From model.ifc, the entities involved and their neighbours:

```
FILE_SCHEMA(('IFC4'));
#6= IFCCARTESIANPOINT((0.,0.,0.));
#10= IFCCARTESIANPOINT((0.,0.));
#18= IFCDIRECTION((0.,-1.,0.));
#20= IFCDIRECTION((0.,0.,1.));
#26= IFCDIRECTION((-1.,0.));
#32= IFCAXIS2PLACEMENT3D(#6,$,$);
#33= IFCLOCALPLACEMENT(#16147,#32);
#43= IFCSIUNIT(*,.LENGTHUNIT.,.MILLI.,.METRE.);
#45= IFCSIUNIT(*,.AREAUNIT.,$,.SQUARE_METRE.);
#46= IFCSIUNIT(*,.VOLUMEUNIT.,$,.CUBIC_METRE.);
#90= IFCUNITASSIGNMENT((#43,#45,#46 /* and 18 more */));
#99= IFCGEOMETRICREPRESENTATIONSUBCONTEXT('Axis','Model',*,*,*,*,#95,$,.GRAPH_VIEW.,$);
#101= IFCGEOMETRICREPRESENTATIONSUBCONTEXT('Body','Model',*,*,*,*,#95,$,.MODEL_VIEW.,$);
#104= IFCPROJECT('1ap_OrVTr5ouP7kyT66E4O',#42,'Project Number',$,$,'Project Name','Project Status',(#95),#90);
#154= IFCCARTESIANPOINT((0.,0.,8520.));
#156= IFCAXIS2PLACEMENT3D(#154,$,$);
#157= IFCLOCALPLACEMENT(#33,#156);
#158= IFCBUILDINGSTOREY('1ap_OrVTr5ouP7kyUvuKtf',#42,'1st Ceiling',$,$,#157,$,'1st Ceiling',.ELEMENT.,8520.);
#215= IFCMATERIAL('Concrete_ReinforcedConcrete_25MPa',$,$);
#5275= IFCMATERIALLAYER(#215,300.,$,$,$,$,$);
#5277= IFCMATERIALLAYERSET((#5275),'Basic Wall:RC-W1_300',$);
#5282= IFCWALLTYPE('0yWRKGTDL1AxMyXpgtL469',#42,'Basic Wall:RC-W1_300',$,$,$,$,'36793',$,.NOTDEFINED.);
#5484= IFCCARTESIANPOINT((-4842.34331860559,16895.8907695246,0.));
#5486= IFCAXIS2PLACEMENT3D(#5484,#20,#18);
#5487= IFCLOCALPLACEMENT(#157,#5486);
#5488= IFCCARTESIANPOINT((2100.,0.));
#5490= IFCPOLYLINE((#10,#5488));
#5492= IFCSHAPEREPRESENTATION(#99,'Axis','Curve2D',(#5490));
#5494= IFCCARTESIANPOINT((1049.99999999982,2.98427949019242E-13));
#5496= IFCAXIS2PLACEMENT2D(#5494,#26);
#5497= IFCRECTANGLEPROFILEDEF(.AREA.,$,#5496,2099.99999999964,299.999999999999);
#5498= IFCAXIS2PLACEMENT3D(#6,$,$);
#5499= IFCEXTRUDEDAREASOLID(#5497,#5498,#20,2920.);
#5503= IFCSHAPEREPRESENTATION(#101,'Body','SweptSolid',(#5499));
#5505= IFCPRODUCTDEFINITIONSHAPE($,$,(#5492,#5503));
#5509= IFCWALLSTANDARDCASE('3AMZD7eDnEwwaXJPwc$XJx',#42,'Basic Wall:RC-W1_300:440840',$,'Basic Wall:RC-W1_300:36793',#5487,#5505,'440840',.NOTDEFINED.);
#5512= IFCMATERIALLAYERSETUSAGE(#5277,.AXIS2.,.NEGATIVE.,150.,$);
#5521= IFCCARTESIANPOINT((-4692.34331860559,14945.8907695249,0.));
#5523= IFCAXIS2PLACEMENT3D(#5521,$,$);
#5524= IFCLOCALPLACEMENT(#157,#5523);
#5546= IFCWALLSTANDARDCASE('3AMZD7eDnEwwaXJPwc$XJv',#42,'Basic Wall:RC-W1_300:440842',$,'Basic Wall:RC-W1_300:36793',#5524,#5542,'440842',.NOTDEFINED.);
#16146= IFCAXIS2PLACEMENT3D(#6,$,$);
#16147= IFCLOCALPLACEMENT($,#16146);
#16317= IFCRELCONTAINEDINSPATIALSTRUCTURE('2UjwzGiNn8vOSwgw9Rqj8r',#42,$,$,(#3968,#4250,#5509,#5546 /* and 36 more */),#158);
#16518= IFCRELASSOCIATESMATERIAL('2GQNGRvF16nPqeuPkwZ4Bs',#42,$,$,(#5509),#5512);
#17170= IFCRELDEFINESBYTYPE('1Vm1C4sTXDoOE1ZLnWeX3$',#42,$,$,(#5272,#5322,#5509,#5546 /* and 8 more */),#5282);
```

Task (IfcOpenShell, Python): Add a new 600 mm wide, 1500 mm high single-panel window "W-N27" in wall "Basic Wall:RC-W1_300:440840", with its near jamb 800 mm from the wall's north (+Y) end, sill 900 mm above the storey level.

```python
import numpy as np
import ifcopenshell
import ifcopenshell.api.feature
import ifcopenshell.api.geometry
import ifcopenshell.api.root
import ifcopenshell.api.spatial
import ifcopenshell.geom
import ifcopenshell.util.element
import ifcopenshell.util.placement
import ifcopenshell.util.representation
import ifcopenshell.util.shape
import ifcopenshell.util.unit

model = ifcopenshell.open("model.ifc")
unit_scale = ifcopenshell.util.unit.calculate_unit_scale(model)
settings = ifcopenshell.geom.settings()


def volume(element):
    """Net volume in cubic metres, openings subtracted."""
    shape = ifcopenshell.geom.create_shape(settings, element)
    return ifcopenshell.util.shape.get_volume(shape.geometry)


wall = model.by_guid("3AMZD7eDnEwwaXJPwc$XJx")
storey = ifcopenshell.util.element.get_container(wall, ifc_class="IfcBuildingStorey")
context = ifcopenshell.util.representation.get_context(model, "Model", "Body", "MODEL_VIEW")
before = volume(wall)

width, height, from_end, sill = 0.6, 1.5, 0.8, 0.9  # metres

# The wall runs along its own X axis, and the end named is its -X end.
wall_shape = ifcopenshell.geom.create_shape(settings, wall)
x, y, z = ifcopenshell.util.shape.get_vertices(wall_shape.geometry).T
start = x.min() + from_end
face, thickness = float(y.min()), float(y.max() - y.min())
wall_matrix = ifcopenshell.util.placement.get_local_placement(wall.ObjectPlacement)
level = ifcopenshell.util.placement.get_local_placement(storey.ObjectPlacement)[2, 3]


def in_wall(x, y):
    """Placement at x, y metres in the wall's axes, at sill height."""
    matrix = wall_matrix.copy()
    matrix[:, 3] = wall_matrix @ np.array([x / unit_scale, y / unit_scale, 0.0, 1.0])
    matrix[2, 3] = level + sill / unit_scale
    return matrix


# Opening: a box that overshoots both wall faces by 50 mm.
opening = ifcopenshell.api.root.create_entity(model, ifc_class="IfcOpeningElement", predefined_type="OPENING")
box = ifcopenshell.api.geometry.add_wall_representation(
    model, context=context, length=width, height=height, thickness=thickness + 0.1
)
ifcopenshell.api.geometry.assign_representation(model, product=opening, representation=box)
ifcopenshell.api.geometry.edit_object_placement(model, product=opening, matrix=in_wall(start, face - 0.05), is_si=False)
ifcopenshell.api.feature.add_feature(model, feature=opening, element=wall)

window = ifcopenshell.api.root.create_entity(model, ifc_class="IfcWindow", name="W-N27", predefined_type="WINDOW")
window.OverallWidth, window.OverallHeight = width / unit_scale, height / unit_scale
window.PartitioningType = "SINGLE_PANEL"
body = ifcopenshell.api.geometry.add_window_representation(
    model,
    context=context,
    overall_width=window.OverallWidth,
    overall_height=window.OverallHeight,
    partition_type="SINGLE_PANEL",
)
ifcopenshell.api.geometry.assign_representation(model, product=window, representation=body)
ifcopenshell.api.spatial.assign_container(model, products=[window], relating_structure=storey)
ifcopenshell.api.feature.add_filling(model, opening=opening, element=window)

# Centre the window in the wall's thickness.
ifcopenshell.api.geometry.edit_object_placement(model, product=window, matrix=in_wall(start, face), is_si=False)
window_shape = ifcopenshell.geom.create_shape(settings, window)
depth = ifcopenshell.util.shape.get_vertices(window_shape.geometry)[:, 1]
offset = face + thickness / 2 - (depth.min() + depth.max()) / 2
ifcopenshell.api.geometry.edit_object_placement(model, product=window, matrix=in_wall(start, offset), is_si=False)

after = volume(wall)

print(f"wall volume {before:.3f} -> {after:.3f} m3")

model.write("model-out.ifc")
```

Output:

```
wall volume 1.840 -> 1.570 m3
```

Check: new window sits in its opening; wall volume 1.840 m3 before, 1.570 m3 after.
